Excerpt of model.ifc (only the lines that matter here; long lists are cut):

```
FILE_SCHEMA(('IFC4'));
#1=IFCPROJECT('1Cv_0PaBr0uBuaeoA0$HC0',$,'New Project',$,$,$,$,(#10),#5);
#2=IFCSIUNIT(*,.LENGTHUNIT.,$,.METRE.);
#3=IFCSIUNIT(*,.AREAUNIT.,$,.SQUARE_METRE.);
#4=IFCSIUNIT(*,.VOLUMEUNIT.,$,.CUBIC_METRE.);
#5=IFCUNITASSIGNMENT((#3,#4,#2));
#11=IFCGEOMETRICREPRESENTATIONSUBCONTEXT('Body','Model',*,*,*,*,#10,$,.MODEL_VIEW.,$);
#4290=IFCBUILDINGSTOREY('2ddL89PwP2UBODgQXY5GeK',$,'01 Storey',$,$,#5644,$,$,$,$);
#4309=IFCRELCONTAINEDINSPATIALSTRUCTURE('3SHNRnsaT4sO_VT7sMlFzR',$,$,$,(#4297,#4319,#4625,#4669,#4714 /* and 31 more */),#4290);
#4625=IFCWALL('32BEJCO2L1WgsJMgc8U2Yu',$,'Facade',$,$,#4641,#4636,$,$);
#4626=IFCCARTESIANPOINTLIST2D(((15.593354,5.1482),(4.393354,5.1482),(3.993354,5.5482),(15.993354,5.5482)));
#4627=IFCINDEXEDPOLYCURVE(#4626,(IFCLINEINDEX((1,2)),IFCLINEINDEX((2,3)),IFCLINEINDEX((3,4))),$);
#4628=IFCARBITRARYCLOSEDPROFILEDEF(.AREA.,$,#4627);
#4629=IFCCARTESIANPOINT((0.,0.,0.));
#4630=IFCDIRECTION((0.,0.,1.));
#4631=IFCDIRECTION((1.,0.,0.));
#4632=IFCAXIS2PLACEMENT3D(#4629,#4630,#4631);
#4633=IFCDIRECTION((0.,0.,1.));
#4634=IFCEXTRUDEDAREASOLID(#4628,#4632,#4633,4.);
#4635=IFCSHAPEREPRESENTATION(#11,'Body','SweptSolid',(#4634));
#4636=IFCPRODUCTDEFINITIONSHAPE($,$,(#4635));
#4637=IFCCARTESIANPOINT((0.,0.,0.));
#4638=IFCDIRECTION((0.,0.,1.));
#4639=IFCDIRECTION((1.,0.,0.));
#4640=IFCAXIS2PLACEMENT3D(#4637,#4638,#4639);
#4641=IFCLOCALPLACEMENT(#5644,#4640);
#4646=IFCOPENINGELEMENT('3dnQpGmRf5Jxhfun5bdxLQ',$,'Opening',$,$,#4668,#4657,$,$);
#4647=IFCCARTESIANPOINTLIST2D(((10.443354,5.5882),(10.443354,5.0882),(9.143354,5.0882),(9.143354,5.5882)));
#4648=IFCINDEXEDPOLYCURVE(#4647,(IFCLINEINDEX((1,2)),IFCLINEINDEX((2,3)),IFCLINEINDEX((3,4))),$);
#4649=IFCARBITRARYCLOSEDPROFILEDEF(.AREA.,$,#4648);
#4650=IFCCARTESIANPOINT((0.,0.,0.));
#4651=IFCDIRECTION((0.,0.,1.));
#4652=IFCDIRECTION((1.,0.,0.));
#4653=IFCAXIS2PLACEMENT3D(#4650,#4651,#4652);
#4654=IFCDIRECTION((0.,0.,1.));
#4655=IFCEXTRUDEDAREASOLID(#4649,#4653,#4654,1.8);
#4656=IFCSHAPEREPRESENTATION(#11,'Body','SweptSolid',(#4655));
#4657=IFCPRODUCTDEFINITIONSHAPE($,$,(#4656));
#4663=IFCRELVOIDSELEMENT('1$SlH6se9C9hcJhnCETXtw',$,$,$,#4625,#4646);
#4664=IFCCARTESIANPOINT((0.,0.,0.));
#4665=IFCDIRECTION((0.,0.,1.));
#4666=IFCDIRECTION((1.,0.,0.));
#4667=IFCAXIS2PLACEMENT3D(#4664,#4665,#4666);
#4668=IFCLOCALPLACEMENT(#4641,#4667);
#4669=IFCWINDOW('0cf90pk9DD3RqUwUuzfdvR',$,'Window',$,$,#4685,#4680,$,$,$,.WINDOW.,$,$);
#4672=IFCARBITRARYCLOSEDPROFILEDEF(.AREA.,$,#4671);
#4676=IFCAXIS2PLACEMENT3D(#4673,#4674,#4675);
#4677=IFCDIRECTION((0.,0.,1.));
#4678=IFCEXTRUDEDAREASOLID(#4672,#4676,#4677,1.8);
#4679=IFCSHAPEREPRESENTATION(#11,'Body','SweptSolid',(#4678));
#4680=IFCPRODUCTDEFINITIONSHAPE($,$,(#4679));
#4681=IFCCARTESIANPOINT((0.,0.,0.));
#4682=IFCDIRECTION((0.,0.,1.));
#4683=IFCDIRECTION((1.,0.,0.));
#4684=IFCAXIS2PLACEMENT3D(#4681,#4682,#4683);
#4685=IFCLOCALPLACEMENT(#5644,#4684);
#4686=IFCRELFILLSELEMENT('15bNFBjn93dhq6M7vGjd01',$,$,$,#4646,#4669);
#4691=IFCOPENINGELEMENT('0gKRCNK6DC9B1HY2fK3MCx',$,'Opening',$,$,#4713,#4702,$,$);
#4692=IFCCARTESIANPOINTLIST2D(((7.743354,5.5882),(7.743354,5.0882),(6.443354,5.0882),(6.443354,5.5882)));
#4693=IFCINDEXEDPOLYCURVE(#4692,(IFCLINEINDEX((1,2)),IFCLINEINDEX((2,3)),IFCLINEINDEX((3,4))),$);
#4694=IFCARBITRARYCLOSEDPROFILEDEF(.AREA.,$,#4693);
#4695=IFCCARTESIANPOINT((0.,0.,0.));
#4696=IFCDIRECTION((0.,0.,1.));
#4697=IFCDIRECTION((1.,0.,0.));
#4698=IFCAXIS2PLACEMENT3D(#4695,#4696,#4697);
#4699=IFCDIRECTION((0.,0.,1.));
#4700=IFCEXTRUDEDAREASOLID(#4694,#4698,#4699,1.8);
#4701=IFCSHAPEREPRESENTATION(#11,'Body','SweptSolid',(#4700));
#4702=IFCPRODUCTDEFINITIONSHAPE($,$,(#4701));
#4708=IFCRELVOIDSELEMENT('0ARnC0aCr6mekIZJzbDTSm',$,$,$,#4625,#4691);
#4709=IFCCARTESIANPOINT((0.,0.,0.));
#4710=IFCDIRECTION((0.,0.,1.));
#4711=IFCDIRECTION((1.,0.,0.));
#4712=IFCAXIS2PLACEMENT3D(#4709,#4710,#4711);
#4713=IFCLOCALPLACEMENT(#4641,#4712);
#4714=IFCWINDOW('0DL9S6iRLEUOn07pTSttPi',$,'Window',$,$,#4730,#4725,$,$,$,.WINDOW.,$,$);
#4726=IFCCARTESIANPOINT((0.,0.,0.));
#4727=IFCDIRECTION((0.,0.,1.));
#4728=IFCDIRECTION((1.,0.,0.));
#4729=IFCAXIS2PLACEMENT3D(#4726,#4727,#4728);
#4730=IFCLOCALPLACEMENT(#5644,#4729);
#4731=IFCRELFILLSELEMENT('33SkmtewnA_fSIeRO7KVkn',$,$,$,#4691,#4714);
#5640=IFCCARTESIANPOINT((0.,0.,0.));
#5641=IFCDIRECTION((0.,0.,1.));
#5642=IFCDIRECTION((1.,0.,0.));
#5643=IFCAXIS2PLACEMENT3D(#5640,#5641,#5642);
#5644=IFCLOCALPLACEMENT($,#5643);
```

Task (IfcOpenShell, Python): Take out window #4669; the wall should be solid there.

```python
import ifcopenshell
import ifcopenshell.api.feature
import ifcopenshell.api.root
import ifcopenshell.geom
import ifcopenshell.util.shape

model = ifcopenshell.open("model.ifc")
settings = ifcopenshell.geom.settings()


def volume(element):
    """Net volume in cubic metres, openings subtracted."""
    shape = ifcopenshell.geom.create_shape(settings, element)
    return ifcopenshell.util.shape.get_volume(shape.geometry)


window = model.by_guid("0cf90pk9DD3RqUwUuzfdvR")
opening = window.FillsVoids[0].RelatingOpeningElement
wall = opening.VoidsElements[0].RelatingBuildingElement
before = volume(wall)

ifcopenshell.api.root.remove_product(model, product=window)
ifcopenshell.api.feature.remove_feature(model, feature=opening)

after = volume(wall)

print(f"wall volume {before:.3f} -> {after:.3f} m3")

model.write("model_edited.ifc")
```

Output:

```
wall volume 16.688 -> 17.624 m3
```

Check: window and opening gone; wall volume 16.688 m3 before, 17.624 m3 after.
